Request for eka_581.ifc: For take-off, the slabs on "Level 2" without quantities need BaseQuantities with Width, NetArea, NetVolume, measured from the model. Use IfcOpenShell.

First a look at what the model holds.

```python
import ifcopenshell
import ifcopenshell.util.element
import ifcopenshell.util.unit

model = ifcopenshell.open("eka_581.ifc")
print(model.schema)
for unit_type in ("LENGTHUNIT", "AREAUNIT", "VOLUMEUNIT"):
    print(unit_type, ifcopenshell.util.unit.calculate_unit_scale(model, unit_type))
storey = next(s for s in model.by_type("IfcBuildingStorey") if s.Name == "Level 2")
slabs = [e for e in ifcopenshell.util.element.get_decomposition(storey) if e.is_a("IfcSlab")]
for e in sorted(slabs, key=lambda e: e.id()):
    print(e.id(), e.is_a(), e.Name, list(ifcopenshell.util.element.get_psets(e, qtos_only=True)), sep=" | ")
```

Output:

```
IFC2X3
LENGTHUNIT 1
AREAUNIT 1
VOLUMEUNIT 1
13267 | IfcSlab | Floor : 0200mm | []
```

```python
import ifcopenshell
import ifcopenshell.api.pset
import ifcopenshell.geom
import ifcopenshell.util.element
import ifcopenshell.util.shape
import ifcopenshell.util.unit

model = ifcopenshell.open("eka_581.ifc")
unit_scale = ifcopenshell.util.unit.calculate_unit_scale(model)
area_scale = ifcopenshell.util.unit.calculate_unit_scale(model, "AREAUNIT")
volume_scale = ifcopenshell.util.unit.calculate_unit_scale(model, "VOLUMEUNIT")
settings = ifcopenshell.geom.settings()

storey = next(s for s in model.by_type("IfcBuildingStorey") if s.Name == "Level 2")
slabs = [e for e in ifcopenshell.util.element.get_decomposition(storey) if e.is_a("IfcSlab")]

for e in sorted(slabs, key=lambda e: e.id()):
    if ifcopenshell.util.element.get_psets(e, qtos_only=True, should_inherit=False):
        continue
    # Geometry comes back in metres, in the element's own axes.
    shape = ifcopenshell.geom.create_shape(settings, e)
    values = {
        "Width": ifcopenshell.util.shape.get_z(shape.geometry) / unit_scale,
        "NetArea": ifcopenshell.util.shape.get_footprint_area(shape.geometry) / area_scale,
        "NetVolume": ifcopenshell.util.shape.get_volume(shape.geometry) / volume_scale,
    }
    qto = ifcopenshell.api.pset.add_qto(model, product=e, name="BaseQuantities")
    ifcopenshell.api.pset.edit_qto(model, qto=qto, properties=values)
    print(e.id(), {k: round(v, 3) for k, v in values.items()})

model.write("eka_581_updated.ifc")
```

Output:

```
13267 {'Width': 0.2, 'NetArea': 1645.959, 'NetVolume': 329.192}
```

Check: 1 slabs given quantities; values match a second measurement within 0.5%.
